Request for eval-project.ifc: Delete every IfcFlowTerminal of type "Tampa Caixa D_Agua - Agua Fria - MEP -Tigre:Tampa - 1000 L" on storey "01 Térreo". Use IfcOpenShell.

First a look at what the model holds.

```python
import ifcopenshell
import ifcopenshell.util.element

model = ifcopenshell.open("eval-project.ifc")
print(model.schema)
storey = next(s for s in model.by_type("IfcBuildingStorey") if s.Name == "01 Térreo")
terminals = [e for e in ifcopenshell.util.element.get_decomposition(storey) if e.is_a("IfcFlowTerminal")]
seen = {}
for e in terminals:
    element_type = ifcopenshell.util.element.get_type(e)
    name = element_type.Name if element_type not in (None, e) else None
    seen[name] = seen.get(name, 0) + 1
for name, count in sorted(seen.items(), key=str):
    print(count, "x", name)
```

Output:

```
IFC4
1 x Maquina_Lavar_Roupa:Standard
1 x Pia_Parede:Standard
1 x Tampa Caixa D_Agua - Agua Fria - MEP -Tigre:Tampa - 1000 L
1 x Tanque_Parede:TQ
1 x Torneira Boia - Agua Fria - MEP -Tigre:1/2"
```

```python
import ifcopenshell
import ifcopenshell.api.root
import ifcopenshell.util.element

model = ifcopenshell.open("eval-project.ifc")

storey = next(s for s in model.by_type("IfcBuildingStorey") if s.Name == "01 Térreo")
terminals = [e for e in ifcopenshell.util.element.get_decomposition(storey) if e.is_a("IfcFlowTerminal")]
targets = [e for e in terminals if (t := ifcopenshell.util.element.get_type(e)) not in (None, e) and t.Name == "Tampa Caixa D_Agua - Agua Fria - MEP -Tigre:Tampa - 1000 L"]

for e in targets:
    ifcopenshell.api.root.remove_product(model, product=e)
print(len(targets), "removed")

model.write("eval-project_v2.ifc")
```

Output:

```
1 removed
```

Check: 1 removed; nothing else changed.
